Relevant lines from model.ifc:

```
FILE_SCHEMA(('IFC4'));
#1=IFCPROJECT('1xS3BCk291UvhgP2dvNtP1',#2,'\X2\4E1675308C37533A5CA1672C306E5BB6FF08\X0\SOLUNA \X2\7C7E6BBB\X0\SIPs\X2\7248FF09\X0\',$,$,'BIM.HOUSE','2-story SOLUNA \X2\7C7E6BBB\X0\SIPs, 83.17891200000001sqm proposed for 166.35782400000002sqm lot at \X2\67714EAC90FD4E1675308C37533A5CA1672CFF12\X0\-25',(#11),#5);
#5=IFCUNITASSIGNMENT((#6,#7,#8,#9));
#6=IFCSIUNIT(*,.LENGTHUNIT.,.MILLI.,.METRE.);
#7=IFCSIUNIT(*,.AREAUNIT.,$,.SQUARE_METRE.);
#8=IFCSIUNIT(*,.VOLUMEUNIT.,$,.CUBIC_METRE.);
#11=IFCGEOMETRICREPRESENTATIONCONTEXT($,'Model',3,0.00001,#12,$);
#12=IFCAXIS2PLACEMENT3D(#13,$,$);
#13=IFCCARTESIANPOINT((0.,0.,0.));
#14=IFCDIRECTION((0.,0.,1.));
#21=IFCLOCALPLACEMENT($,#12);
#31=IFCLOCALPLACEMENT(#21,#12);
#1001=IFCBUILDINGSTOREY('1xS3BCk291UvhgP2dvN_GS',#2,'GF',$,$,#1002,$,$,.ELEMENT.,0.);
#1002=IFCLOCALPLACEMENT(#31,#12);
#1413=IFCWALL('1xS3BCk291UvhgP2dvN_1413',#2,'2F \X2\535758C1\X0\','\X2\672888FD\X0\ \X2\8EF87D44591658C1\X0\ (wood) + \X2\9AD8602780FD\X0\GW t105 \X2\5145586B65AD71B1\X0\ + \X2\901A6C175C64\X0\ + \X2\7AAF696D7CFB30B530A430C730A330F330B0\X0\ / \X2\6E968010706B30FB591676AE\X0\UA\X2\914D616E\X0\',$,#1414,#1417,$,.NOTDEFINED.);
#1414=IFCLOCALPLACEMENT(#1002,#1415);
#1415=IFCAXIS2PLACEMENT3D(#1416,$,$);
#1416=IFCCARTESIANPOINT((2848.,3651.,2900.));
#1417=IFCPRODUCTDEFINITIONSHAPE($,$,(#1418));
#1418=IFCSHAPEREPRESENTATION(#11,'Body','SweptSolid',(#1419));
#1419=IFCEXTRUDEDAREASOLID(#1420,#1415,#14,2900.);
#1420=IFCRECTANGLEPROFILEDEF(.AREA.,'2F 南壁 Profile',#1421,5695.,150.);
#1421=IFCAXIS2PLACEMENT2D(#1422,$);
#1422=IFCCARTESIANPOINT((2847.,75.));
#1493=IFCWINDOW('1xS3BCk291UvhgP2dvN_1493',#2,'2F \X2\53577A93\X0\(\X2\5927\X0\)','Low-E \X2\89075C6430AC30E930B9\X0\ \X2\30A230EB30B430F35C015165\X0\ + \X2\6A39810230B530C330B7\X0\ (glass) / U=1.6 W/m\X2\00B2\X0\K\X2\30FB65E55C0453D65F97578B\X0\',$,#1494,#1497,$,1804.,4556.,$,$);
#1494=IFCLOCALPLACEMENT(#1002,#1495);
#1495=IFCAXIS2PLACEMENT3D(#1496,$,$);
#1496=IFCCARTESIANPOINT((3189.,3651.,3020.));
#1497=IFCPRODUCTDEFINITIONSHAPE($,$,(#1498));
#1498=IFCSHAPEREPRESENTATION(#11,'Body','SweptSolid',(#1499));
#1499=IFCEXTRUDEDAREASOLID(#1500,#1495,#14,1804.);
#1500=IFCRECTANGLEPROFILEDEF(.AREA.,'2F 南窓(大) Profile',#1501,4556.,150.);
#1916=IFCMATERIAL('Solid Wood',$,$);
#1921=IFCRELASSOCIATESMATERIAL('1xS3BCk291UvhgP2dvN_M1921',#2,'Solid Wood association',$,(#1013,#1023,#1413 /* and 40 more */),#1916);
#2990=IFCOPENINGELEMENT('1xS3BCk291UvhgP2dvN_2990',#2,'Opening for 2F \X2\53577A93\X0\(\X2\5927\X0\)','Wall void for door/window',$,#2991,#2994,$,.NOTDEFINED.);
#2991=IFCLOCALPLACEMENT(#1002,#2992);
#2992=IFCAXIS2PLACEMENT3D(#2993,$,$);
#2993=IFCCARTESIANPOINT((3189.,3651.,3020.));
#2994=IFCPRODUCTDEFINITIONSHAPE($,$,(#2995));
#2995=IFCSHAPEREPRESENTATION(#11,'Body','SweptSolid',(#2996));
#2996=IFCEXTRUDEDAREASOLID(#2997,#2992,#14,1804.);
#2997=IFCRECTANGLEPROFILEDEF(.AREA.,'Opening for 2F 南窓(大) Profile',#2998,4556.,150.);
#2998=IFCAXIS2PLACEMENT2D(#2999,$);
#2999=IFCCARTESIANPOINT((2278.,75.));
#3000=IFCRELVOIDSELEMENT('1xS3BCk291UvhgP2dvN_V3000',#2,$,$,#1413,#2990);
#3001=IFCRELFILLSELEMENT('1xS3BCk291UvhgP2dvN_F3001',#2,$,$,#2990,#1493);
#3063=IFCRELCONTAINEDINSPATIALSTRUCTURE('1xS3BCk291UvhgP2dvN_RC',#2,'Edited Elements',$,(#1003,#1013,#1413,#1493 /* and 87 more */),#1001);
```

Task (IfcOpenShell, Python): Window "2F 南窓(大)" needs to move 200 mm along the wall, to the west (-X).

```python
import ifcopenshell
import ifcopenshell.api.geometry
import ifcopenshell.util.placement

model = ifcopenshell.open("model.ifc")

window = model.by_guid("1xS3BCk291UvhgP2dvN_1493")
opening = window.FillsVoids[0].RelatingOpeningElement
wall = opening.VoidsElements[0].RelatingBuildingElement

wall_matrix = ifcopenshell.util.placement.get_local_placement(wall.ObjectPlacement)
shift = wall_matrix[:3, 0] * -200.0
before = ifcopenshell.util.placement.get_local_placement(window.ObjectPlacement)[:3, 3].copy()

# The window is not placed relative to its opening, so move both.
for product in (opening, window):
    matrix = ifcopenshell.util.placement.get_local_placement(product.ObjectPlacement)
    matrix[:3, 3] += shift
    ifcopenshell.api.geometry.edit_object_placement(model, product=product, matrix=matrix, is_si=False)

after = ifcopenshell.util.placement.get_local_placement(window.ObjectPlacement)[:3, 3]
print("window moved by", (after - before).round(3) + 0.0)

model.write("model_edited.ifc")
```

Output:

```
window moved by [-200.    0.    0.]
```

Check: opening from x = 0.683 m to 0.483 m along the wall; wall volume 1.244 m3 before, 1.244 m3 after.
